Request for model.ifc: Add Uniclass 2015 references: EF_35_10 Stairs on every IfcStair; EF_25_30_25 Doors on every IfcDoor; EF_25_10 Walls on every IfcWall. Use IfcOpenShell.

First a look at what the model holds.

```python
import ifcopenshell

model = ifcopenshell.open("model.ifc")
print(model.schema)
print("classifications:", [c.Name for c in model.by_type("IfcClassification")])
for ifc_class in ("IfcDoor", "IfcRoof", "IfcStair", "IfcWall", "IfcWindow"):
    print(ifc_class, len(model.by_type(ifc_class)))
```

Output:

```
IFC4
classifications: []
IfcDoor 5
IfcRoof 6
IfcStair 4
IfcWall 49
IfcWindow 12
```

```python
import ifcopenshell
import ifcopenshell.api.classification

model = ifcopenshell.open("model.ifc")

system = ifcopenshell.api.classification.add_classification(model, classification="Uniclass 2015")

codes = {
    "IfcStair": ("EF_35_10", "Stairs"),
    "IfcDoor": ("EF_25_30_25", "Doors"),
    "IfcWall": ("EF_25_10", "Walls"),
}
for ifc_class, (code, name) in codes.items():
    products = model.by_type(ifc_class)
    ifcopenshell.api.classification.add_reference(
        model, products=products, classification=system, identification=code, name=name
    )
    print(code, len(products))

model.write("model_v2.ifc")
```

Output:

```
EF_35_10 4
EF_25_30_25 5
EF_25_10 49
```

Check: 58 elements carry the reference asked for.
